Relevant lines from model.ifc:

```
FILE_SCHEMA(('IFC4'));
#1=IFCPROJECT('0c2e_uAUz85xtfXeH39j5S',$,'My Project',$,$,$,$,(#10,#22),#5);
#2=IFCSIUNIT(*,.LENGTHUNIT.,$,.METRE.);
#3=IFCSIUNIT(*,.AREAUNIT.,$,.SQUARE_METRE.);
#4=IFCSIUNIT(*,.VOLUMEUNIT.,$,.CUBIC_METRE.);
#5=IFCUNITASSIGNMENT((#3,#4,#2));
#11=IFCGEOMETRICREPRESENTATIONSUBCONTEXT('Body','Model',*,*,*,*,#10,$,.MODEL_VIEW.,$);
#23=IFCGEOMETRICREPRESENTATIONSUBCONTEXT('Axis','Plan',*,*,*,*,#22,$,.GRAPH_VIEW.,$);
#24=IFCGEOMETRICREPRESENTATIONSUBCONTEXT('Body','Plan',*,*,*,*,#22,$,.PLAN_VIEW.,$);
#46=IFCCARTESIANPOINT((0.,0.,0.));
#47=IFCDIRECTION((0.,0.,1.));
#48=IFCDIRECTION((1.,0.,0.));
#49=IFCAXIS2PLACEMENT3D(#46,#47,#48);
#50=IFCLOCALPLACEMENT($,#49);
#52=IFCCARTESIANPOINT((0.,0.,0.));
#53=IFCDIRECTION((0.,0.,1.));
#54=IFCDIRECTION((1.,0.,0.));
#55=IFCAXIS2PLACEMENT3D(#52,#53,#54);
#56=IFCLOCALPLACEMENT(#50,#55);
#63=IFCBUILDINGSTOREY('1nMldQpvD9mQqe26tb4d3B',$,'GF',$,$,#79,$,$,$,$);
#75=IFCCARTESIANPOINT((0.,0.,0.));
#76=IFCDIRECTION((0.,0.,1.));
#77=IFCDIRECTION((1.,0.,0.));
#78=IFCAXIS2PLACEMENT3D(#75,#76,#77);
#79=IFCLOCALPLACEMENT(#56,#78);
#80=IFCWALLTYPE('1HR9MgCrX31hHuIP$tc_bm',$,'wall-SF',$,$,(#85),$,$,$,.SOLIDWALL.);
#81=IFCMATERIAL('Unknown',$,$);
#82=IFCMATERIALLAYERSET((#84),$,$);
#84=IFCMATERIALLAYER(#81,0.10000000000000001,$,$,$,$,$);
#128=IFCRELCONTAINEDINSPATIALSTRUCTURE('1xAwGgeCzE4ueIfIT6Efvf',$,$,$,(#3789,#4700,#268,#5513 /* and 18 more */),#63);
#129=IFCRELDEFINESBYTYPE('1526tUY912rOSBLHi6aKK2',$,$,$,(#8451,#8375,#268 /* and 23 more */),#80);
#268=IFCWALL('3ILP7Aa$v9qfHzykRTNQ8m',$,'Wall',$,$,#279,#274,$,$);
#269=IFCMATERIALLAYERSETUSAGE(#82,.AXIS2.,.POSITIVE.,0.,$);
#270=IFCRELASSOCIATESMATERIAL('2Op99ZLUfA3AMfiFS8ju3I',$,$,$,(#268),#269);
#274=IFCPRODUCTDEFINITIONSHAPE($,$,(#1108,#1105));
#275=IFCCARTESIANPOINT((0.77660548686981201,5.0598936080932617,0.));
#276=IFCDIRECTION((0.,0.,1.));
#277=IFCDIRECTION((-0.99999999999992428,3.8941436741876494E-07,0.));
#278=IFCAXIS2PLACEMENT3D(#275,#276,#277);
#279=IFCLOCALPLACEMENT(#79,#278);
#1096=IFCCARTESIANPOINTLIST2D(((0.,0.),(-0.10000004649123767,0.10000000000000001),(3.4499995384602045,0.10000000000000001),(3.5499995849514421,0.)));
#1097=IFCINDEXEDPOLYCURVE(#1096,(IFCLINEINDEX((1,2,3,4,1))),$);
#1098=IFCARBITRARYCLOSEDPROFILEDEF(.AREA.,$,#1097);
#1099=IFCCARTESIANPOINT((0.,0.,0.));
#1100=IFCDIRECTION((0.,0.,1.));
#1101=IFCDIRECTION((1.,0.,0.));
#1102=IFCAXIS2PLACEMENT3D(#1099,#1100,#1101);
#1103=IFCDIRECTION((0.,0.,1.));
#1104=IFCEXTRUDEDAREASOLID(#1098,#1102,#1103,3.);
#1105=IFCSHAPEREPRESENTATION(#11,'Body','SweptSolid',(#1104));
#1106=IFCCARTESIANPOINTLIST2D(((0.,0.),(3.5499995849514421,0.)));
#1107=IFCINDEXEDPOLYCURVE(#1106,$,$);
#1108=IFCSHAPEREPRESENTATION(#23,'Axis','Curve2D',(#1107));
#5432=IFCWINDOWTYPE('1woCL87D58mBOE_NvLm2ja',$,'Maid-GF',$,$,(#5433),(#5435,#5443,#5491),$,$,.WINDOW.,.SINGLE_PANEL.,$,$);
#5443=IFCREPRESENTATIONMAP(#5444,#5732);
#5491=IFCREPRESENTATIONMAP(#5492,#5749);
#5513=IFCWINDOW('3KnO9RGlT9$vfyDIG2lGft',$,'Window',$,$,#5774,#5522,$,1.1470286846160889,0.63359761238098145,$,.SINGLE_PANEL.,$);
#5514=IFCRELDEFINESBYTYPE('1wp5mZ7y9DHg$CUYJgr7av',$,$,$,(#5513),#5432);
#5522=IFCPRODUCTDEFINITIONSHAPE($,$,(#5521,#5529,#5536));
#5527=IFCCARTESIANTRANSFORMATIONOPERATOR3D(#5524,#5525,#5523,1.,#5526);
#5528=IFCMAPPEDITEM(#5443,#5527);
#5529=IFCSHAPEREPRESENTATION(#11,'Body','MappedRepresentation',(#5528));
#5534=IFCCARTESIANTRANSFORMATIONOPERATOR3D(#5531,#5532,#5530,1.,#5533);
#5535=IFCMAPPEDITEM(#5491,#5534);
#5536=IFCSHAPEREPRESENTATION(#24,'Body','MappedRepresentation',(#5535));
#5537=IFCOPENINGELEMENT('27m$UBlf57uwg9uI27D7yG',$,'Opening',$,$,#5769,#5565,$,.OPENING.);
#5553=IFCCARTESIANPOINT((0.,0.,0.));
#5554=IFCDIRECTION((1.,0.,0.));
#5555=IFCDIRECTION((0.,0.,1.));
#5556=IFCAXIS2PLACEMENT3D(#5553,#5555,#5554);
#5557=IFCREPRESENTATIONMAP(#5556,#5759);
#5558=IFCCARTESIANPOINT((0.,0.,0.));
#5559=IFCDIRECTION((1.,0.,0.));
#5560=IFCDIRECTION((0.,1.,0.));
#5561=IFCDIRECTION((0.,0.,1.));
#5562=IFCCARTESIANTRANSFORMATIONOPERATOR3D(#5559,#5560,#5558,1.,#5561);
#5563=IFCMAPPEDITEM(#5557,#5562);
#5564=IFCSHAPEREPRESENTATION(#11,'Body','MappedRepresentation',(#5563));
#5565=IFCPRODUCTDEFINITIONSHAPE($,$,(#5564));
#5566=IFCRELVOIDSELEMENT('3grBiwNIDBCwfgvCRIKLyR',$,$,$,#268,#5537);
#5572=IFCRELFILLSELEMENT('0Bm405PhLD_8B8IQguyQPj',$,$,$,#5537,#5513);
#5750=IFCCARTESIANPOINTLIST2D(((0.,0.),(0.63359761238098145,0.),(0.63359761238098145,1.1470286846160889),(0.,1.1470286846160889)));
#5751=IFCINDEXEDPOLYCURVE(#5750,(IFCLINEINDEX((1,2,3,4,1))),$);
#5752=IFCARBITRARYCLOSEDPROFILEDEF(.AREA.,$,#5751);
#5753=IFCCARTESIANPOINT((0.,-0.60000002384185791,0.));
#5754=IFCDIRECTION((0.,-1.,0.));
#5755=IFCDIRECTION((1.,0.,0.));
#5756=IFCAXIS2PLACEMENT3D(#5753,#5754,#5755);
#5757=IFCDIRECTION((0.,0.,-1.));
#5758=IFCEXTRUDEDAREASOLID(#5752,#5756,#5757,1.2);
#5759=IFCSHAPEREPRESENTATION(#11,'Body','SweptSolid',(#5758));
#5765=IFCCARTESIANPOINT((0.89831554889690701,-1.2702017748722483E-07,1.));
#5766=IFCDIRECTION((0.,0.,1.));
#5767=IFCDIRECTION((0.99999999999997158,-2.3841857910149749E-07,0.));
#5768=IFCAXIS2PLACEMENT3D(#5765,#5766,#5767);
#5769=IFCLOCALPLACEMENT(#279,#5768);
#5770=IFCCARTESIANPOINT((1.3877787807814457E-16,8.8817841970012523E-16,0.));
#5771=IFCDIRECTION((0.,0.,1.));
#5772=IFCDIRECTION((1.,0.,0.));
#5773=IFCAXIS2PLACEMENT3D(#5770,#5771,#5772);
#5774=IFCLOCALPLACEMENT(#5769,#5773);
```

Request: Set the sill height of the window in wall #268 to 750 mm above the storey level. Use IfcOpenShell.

```python
import numpy as np
import ifcopenshell
import ifcopenshell.api.geometry
import ifcopenshell.geom
import ifcopenshell.util.element
import ifcopenshell.util.placement
import ifcopenshell.util.shape
import ifcopenshell.util.unit

model = ifcopenshell.open("model.ifc")
unit_scale = ifcopenshell.util.unit.calculate_unit_scale(model)

window = model.by_id(5513)
opening = window.FillsVoids[0].RelatingOpeningElement
storey = ifcopenshell.util.element.get_container(window, ifc_class="IfcBuildingStorey")
level = ifcopenshell.util.placement.get_local_placement(storey.ObjectPlacement)[2, 3]

# The opening's origin need not be at the sill, so measure its lowest point.
shape = ifcopenshell.geom.create_shape(ifcopenshell.geom.settings(), opening)
bottom = ifcopenshell.util.shape.get_shape_bottom_elevation(shape, shape.geometry) / unit_scale
dz = level + 0.75 / unit_scale - bottom

shift = np.array([0.0, 0.0, dz])
# The window is placed relative to its opening, so it follows when the opening moves.
matrix = ifcopenshell.util.placement.get_local_placement(opening.ObjectPlacement)
matrix[:3, 3] += shift
ifcopenshell.api.geometry.edit_object_placement(
    model, product=opening, matrix=matrix, is_si=False, should_transform_children=True
)

print(f"moved by {dz * unit_scale:+.3f} m")

model.write("model_v2.ifc")
```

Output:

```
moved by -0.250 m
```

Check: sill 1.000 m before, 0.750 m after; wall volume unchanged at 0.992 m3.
